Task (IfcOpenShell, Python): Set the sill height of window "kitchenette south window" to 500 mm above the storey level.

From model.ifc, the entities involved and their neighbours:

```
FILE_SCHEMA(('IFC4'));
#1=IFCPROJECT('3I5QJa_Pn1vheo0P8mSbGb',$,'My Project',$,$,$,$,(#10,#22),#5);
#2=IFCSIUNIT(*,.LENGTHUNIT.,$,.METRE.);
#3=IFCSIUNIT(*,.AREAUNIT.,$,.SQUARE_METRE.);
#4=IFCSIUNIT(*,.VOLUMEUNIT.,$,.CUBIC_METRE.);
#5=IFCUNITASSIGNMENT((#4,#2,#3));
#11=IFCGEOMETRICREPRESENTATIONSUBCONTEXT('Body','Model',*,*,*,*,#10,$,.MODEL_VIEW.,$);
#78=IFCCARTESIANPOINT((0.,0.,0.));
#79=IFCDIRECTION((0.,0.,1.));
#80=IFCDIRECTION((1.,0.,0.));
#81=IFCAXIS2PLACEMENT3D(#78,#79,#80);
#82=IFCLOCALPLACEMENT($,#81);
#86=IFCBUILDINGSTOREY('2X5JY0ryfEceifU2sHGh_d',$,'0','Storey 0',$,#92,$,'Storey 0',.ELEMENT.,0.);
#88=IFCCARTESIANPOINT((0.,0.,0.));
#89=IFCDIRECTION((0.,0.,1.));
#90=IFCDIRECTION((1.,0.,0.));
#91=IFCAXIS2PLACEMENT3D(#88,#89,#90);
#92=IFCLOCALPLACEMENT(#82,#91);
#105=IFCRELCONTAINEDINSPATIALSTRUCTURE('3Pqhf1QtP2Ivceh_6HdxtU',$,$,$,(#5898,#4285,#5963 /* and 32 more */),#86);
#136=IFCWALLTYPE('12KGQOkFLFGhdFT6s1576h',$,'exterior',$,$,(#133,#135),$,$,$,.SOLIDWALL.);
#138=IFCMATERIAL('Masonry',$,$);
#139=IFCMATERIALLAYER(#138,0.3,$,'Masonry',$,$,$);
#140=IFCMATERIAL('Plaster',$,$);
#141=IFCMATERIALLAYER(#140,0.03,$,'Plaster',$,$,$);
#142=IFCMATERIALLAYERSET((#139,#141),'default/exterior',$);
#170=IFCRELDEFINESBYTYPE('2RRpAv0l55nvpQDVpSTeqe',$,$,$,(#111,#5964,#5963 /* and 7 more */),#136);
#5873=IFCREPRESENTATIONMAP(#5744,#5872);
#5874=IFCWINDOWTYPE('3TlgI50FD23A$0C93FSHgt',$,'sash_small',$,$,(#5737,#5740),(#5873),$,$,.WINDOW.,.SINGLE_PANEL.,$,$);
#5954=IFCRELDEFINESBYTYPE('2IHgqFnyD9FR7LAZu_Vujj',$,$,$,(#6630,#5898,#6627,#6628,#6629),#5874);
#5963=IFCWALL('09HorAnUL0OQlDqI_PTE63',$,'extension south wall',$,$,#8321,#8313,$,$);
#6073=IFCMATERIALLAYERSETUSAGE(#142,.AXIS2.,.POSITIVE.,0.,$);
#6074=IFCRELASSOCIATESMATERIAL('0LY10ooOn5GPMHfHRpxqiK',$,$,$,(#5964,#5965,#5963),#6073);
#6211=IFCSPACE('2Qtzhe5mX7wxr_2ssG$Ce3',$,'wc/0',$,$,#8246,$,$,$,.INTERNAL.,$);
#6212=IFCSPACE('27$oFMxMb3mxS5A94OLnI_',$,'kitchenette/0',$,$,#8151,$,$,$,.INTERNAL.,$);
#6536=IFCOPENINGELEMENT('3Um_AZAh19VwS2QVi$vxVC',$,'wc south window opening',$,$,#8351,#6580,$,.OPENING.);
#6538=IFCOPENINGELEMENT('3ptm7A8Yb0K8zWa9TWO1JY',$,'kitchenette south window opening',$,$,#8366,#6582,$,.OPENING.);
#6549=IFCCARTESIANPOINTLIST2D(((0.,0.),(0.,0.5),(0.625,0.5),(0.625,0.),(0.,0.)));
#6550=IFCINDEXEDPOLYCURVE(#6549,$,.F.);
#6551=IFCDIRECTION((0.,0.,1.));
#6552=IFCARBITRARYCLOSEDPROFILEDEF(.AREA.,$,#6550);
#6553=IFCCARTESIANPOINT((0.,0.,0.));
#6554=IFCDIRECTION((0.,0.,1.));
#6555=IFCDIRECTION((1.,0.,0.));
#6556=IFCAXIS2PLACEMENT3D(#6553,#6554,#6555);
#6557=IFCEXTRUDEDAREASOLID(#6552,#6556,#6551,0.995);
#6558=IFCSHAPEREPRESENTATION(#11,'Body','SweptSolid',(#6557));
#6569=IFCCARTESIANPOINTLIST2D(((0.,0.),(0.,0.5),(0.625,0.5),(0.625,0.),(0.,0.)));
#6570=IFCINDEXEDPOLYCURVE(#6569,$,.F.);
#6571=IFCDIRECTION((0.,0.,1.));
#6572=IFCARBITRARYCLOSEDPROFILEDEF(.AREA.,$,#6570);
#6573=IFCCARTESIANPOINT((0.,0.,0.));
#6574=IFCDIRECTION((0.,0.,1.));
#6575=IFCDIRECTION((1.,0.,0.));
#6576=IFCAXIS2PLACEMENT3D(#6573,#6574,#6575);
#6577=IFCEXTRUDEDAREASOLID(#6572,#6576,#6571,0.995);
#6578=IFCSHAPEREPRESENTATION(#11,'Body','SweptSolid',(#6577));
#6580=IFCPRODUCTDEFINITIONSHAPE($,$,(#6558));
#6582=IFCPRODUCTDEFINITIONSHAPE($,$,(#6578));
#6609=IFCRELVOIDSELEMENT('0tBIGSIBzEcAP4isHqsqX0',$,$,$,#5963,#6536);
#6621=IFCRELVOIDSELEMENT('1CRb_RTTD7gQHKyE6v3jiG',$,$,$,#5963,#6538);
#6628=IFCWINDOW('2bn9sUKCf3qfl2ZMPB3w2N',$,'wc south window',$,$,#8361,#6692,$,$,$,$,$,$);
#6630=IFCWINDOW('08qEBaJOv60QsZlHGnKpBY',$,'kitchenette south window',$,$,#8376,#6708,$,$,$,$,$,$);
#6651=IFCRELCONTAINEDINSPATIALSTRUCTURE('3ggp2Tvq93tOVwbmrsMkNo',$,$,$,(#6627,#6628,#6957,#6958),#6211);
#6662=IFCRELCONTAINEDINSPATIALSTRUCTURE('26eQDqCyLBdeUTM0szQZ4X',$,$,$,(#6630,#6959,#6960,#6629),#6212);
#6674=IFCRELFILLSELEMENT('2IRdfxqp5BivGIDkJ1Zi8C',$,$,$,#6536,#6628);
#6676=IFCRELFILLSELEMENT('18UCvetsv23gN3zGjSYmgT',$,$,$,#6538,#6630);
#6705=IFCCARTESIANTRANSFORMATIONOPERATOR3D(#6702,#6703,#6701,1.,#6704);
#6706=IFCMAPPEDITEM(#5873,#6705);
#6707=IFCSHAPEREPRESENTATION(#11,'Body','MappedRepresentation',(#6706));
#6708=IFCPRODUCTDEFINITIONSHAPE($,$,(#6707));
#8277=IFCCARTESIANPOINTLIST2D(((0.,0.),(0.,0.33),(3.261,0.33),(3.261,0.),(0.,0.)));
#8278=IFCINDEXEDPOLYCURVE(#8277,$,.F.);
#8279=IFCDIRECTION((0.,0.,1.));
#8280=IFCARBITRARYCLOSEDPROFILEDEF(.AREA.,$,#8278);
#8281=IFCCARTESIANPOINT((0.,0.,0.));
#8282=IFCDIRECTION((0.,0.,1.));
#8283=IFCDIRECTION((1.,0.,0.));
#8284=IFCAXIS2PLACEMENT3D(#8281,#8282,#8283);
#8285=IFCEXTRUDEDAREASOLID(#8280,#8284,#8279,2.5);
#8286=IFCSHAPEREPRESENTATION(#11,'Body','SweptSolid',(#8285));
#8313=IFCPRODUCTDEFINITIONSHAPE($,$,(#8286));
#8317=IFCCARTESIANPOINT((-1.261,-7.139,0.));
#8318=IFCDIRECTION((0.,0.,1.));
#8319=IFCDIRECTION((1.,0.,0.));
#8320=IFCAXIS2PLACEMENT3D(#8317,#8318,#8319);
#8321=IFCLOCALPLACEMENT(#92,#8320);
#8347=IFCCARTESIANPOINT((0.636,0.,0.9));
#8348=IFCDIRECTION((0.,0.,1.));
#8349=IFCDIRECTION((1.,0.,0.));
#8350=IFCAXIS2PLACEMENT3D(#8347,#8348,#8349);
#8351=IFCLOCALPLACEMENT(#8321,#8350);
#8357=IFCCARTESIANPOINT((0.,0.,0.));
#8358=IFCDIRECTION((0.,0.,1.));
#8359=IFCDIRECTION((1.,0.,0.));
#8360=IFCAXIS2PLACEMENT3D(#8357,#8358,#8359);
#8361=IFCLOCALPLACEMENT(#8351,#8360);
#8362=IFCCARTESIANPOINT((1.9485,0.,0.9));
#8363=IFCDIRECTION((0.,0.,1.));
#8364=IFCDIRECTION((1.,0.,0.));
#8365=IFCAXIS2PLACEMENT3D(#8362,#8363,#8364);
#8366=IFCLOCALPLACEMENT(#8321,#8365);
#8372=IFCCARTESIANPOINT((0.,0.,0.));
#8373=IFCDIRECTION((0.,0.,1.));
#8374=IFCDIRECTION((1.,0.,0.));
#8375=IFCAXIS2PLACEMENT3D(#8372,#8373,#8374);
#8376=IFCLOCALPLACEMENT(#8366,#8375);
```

```python
import numpy as np
import ifcopenshell
import ifcopenshell.api.geometry
import ifcopenshell.geom
import ifcopenshell.util.element
import ifcopenshell.util.placement
import ifcopenshell.util.shape
import ifcopenshell.util.unit

model = ifcopenshell.open("model.ifc")
unit_scale = ifcopenshell.util.unit.calculate_unit_scale(model)

window = model.by_guid("08qEBaJOv60QsZlHGnKpBY")
opening = window.FillsVoids[0].RelatingOpeningElement
storey = ifcopenshell.util.element.get_container(window, ifc_class="IfcBuildingStorey")
level = ifcopenshell.util.placement.get_local_placement(storey.ObjectPlacement)[2, 3]

# The opening's origin need not be at the sill, so measure its lowest point.
shape = ifcopenshell.geom.create_shape(ifcopenshell.geom.settings(), opening)
bottom = ifcopenshell.util.shape.get_shape_bottom_elevation(shape, shape.geometry) / unit_scale
dz = level + 0.5 - bottom

shift = np.array([0.0, 0.0, dz])
# The window is placed relative to its opening, so it follows when the opening moves.
matrix = ifcopenshell.util.placement.get_local_placement(opening.ObjectPlacement)
matrix[:3, 3] += shift
ifcopenshell.api.geometry.edit_object_placement(
    model, product=opening, matrix=matrix, is_si=False, should_transform_children=True
)

print(f"moved by {dz * unit_scale:+.3f} m")

model.write("model_v2.ifc")
```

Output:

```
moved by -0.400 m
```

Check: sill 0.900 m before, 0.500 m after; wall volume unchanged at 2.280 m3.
